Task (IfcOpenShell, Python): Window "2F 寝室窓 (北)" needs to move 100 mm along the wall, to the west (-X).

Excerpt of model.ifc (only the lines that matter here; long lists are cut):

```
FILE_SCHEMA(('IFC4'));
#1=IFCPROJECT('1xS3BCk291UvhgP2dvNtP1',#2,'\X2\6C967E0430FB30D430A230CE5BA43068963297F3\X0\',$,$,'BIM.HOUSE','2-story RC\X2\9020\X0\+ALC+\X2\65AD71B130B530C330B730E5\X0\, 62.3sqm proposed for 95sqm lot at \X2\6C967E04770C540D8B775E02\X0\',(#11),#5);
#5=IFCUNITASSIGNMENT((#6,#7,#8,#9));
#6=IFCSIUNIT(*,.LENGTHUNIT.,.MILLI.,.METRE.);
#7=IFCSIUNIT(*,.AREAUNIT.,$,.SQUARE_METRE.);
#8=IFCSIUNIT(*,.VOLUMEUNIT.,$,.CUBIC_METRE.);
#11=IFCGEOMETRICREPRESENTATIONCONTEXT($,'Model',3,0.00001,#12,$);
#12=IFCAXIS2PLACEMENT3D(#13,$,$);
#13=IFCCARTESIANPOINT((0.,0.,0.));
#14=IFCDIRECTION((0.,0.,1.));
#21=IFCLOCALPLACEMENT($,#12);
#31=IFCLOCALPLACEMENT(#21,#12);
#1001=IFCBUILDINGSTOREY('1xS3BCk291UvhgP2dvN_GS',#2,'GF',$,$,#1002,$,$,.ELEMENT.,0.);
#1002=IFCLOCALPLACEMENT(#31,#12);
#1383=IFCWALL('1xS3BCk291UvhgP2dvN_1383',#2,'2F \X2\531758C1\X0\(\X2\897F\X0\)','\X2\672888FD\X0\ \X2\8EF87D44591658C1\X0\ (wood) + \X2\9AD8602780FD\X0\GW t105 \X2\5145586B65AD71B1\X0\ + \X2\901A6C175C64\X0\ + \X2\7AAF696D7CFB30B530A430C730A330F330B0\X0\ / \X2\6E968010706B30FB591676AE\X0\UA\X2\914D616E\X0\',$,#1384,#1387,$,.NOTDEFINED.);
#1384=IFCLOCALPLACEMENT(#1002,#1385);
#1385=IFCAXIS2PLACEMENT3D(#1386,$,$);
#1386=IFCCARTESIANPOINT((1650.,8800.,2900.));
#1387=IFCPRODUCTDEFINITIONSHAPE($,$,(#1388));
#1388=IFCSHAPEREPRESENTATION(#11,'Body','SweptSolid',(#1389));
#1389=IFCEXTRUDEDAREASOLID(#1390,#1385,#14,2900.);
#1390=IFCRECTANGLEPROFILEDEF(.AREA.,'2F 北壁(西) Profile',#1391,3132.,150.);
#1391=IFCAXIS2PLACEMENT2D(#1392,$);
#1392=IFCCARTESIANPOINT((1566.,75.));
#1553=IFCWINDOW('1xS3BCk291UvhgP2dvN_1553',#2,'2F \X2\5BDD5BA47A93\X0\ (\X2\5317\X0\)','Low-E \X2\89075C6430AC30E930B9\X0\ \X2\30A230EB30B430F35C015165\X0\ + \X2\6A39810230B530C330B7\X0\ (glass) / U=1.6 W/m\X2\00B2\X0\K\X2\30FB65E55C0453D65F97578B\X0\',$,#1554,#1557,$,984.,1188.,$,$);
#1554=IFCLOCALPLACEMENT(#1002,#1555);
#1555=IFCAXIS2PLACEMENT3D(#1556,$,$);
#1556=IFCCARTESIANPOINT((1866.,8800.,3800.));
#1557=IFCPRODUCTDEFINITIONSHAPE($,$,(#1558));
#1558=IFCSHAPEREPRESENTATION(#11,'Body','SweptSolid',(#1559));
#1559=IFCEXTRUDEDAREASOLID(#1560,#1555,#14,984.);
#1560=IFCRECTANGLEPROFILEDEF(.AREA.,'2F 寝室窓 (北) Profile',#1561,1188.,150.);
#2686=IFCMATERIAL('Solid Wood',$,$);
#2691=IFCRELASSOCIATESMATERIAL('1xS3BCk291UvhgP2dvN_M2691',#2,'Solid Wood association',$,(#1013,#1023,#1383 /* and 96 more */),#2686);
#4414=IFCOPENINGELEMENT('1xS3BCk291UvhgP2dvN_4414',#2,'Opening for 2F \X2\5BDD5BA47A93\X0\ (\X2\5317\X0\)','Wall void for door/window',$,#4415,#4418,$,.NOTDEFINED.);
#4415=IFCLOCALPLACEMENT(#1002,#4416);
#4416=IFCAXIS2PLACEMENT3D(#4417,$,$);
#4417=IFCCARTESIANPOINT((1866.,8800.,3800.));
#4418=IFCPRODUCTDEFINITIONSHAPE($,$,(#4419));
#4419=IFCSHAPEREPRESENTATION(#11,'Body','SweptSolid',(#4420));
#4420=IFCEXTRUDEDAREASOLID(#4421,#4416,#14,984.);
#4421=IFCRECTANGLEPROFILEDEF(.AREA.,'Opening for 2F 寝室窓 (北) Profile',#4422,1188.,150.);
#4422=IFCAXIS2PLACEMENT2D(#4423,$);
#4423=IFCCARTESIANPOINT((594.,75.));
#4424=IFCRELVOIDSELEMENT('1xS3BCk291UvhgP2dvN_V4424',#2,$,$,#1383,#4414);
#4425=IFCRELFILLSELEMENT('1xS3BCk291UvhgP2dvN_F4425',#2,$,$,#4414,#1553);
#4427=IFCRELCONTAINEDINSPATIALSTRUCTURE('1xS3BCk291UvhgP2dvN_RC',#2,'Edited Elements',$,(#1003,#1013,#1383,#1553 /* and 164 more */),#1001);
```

```python
import ifcopenshell
import ifcopenshell.api.geometry
import ifcopenshell.util.placement
import ifcopenshell.util.unit

model = ifcopenshell.open("model.ifc")
unit_scale = ifcopenshell.util.unit.calculate_unit_scale(model)

window = model.by_guid("1xS3BCk291UvhgP2dvN_1553")
opening = window.FillsVoids[0].RelatingOpeningElement
wall = opening.VoidsElements[0].RelatingBuildingElement

wall_matrix = ifcopenshell.util.placement.get_local_placement(wall.ObjectPlacement)
shift = wall_matrix[:3, 0] * -0.1 / unit_scale
before = ifcopenshell.util.placement.get_local_placement(window.ObjectPlacement)[:3, 3].copy()

# The window is not placed relative to its opening, so move both.
for product in (opening, window):
    matrix = ifcopenshell.util.placement.get_local_placement(product.ObjectPlacement)
    matrix[:3, 3] += shift
    ifcopenshell.api.geometry.edit_object_placement(model, product=product, matrix=matrix, is_si=False)

after = ifcopenshell.util.placement.get_local_placement(window.ObjectPlacement)[:3, 3]
print("window moved by", (after - before).round(3) + 0.0)

model.write("model_edited.ifc")
```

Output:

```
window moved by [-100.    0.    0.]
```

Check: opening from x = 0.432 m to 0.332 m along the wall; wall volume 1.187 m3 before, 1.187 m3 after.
